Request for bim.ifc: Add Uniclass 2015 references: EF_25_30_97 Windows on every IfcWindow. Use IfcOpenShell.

First a look at what the model holds.

```python
import ifcopenshell

model = ifcopenshell.open("bim.ifc")
print(model.schema)
print("classifications:", [c.Name for c in model.by_type("IfcClassification")])
for ifc_class in ("IfcDoor", "IfcRoof", "IfcStair", "IfcWall", "IfcWindow"):
    print(ifc_class, len(model.by_type(ifc_class)))
```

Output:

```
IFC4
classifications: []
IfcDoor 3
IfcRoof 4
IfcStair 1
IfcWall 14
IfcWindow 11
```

```python
import ifcopenshell
import ifcopenshell.api.classification

model = ifcopenshell.open("bim.ifc")

system = ifcopenshell.api.classification.add_classification(model, classification="Uniclass 2015")

codes = {
    "IfcWindow": ("EF_25_30_97", "Windows"),
}
for ifc_class, (code, name) in codes.items():
    products = model.by_type(ifc_class)
    ifcopenshell.api.classification.add_reference(
        model, products=products, classification=system, identification=code, name=name
    )
    print(code, len(products))

model.write("bim_updated.ifc")
```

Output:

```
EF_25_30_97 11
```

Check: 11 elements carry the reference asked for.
